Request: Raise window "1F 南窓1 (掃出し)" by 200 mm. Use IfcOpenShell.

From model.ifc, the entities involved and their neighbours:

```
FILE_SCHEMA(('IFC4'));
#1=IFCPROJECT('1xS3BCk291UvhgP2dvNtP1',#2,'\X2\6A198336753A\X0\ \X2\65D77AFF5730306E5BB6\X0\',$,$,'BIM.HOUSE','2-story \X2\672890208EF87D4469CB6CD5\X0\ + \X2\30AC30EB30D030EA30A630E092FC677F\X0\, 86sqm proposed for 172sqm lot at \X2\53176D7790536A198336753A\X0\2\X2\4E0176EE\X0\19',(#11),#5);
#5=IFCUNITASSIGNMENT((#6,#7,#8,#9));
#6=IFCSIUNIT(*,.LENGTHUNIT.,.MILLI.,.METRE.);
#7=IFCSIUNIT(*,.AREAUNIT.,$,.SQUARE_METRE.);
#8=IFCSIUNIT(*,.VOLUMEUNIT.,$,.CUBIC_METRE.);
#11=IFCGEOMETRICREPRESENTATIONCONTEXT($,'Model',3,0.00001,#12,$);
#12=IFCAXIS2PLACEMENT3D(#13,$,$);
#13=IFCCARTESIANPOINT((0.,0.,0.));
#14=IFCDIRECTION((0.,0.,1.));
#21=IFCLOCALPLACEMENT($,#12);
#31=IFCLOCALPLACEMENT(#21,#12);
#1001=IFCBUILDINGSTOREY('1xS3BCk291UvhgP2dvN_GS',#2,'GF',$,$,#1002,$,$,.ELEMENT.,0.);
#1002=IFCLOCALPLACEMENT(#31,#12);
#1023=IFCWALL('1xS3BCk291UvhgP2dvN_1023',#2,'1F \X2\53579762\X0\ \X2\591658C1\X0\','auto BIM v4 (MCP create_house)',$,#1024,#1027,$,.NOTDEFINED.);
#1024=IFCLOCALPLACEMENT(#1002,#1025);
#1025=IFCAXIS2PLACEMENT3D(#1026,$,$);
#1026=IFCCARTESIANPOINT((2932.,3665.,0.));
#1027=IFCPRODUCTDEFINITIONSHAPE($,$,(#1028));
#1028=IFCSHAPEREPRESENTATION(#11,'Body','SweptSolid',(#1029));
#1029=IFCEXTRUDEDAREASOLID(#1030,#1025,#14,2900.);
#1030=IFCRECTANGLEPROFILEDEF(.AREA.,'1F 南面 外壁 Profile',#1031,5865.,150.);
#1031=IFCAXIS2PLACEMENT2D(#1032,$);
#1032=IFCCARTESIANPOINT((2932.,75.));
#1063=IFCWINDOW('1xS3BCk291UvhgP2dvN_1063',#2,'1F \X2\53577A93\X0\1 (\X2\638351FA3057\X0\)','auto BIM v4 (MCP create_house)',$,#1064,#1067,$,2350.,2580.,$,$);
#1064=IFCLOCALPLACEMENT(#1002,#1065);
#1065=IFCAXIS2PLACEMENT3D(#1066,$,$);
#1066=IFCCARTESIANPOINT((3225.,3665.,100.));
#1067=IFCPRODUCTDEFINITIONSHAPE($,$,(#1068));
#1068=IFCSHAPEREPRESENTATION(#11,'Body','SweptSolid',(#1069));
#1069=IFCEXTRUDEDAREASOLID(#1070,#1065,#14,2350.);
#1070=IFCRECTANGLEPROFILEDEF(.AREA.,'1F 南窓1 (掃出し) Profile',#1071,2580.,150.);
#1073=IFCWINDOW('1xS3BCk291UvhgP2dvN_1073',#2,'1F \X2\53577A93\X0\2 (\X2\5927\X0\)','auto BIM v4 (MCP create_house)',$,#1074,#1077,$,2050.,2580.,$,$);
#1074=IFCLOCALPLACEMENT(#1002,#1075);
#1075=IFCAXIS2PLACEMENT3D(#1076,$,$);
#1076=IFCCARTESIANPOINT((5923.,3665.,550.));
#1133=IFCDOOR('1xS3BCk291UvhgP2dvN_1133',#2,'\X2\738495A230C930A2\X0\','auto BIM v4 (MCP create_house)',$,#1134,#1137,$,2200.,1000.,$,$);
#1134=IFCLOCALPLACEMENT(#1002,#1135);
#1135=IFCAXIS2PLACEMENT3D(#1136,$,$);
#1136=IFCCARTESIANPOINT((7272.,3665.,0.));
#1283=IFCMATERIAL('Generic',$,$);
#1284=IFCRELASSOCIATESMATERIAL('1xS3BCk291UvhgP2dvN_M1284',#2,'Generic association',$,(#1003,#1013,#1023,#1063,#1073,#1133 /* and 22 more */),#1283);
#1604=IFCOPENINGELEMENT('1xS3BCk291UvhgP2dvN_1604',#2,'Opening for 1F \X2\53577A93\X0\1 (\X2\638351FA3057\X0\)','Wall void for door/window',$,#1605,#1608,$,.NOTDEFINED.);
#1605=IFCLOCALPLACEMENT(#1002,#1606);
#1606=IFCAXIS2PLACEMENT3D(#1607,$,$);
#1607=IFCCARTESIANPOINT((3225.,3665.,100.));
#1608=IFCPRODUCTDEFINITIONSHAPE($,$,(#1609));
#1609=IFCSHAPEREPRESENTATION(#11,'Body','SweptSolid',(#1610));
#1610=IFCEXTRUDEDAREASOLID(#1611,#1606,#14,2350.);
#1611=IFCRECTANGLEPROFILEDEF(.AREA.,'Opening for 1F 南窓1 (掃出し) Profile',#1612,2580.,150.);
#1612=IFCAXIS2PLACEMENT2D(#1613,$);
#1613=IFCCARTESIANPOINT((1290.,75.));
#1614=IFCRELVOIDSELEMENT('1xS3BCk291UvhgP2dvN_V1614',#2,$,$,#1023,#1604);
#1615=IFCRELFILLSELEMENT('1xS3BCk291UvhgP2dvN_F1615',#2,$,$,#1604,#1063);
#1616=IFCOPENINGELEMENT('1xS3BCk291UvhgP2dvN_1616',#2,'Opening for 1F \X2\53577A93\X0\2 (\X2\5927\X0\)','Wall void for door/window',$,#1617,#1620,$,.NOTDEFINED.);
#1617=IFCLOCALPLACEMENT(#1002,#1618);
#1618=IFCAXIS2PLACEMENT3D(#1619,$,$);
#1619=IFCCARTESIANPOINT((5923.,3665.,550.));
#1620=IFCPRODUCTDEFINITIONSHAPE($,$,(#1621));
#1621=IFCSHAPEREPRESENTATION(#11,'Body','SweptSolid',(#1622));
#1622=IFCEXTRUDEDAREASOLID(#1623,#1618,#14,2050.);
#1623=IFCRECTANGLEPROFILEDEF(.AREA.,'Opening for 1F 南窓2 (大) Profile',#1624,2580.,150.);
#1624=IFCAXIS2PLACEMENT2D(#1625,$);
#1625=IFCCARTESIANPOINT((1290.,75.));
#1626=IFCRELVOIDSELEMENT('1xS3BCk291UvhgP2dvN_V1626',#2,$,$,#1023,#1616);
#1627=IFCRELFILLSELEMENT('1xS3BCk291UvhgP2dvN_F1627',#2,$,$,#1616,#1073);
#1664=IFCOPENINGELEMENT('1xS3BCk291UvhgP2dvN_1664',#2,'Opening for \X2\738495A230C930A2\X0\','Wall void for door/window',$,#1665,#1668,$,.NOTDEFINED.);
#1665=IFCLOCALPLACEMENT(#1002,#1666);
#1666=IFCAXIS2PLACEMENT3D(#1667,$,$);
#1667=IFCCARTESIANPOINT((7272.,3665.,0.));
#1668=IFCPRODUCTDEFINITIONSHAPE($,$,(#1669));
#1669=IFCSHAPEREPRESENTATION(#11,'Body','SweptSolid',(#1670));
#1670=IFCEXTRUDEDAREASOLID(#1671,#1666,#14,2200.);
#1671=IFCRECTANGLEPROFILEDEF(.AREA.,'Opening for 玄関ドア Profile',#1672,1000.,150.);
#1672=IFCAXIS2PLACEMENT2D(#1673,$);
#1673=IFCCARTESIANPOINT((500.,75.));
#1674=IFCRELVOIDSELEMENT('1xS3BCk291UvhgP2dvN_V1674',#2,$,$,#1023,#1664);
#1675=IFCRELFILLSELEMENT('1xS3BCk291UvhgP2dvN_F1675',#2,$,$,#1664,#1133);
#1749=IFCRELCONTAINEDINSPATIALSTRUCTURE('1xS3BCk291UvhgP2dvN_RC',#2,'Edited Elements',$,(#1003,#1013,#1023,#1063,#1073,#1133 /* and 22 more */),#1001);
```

```python
import numpy as np
import ifcopenshell
import ifcopenshell.api.geometry
import ifcopenshell.util.placement
import ifcopenshell.util.unit

model = ifcopenshell.open("model.ifc")
unit_scale = ifcopenshell.util.unit.calculate_unit_scale(model)

window = model.by_guid("1xS3BCk291UvhgP2dvN_1063")
opening = window.FillsVoids[0].RelatingOpeningElement
dz = 0.2 / unit_scale

shift = np.array([0.0, 0.0, dz])
# The window is not placed relative to its opening, so move both.
for product in (opening, window):
    matrix = ifcopenshell.util.placement.get_local_placement(product.ObjectPlacement)
    matrix[:3, 3] += shift
    ifcopenshell.api.geometry.edit_object_placement(model, product=product, matrix=matrix, is_si=False)

print(f"moved by {dz * unit_scale:+.3f} m")

model.write("model_updated.ifc")
```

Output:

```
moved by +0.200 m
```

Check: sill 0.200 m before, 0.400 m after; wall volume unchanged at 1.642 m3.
